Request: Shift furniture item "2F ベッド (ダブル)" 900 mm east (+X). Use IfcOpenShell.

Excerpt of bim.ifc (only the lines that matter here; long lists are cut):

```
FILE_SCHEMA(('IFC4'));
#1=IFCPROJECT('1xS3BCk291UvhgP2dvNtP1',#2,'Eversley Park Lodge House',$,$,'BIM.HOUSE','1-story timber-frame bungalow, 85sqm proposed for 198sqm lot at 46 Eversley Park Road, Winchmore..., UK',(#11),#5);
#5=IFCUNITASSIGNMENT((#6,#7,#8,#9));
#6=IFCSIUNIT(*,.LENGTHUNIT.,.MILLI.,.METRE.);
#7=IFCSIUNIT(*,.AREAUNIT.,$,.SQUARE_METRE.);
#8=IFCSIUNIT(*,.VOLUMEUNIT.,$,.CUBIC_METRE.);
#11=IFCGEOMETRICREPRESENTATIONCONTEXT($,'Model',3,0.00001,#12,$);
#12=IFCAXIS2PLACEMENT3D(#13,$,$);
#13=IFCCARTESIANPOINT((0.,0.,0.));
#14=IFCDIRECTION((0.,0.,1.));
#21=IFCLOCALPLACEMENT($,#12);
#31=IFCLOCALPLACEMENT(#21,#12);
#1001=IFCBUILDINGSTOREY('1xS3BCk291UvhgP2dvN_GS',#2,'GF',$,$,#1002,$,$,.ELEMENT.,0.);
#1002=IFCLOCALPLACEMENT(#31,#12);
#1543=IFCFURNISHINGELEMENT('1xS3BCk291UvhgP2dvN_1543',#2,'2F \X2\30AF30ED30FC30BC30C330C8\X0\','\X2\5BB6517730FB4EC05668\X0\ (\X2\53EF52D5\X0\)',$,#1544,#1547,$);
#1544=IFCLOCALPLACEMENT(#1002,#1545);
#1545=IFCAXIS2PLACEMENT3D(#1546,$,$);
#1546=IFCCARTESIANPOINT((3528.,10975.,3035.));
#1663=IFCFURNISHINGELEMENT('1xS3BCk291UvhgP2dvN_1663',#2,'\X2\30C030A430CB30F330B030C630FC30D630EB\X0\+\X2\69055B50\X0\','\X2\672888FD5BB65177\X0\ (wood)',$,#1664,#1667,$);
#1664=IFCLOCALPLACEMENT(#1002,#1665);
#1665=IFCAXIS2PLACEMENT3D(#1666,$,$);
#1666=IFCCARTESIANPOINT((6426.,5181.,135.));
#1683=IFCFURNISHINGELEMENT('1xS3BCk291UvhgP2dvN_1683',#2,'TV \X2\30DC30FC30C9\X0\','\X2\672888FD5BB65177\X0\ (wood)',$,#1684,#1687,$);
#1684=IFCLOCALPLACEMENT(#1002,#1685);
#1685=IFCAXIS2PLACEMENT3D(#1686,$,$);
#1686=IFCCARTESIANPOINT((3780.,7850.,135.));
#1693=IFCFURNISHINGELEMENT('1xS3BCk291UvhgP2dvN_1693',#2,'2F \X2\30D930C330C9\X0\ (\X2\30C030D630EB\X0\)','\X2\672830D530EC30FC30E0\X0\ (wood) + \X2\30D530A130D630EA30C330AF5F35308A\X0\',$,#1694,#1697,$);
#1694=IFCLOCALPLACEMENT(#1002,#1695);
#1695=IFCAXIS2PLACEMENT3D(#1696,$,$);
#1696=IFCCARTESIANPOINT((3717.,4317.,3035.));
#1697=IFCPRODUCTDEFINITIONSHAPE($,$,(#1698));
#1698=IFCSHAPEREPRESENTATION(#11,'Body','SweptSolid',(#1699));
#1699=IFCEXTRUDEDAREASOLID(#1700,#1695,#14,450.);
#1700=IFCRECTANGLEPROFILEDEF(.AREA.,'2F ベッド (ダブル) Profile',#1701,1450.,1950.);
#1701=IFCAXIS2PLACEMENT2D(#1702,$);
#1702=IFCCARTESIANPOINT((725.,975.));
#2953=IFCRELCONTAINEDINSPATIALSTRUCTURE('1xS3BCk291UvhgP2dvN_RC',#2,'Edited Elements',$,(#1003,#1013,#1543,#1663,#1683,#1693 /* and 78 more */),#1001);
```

```python
import ifcopenshell
import ifcopenshell.api.geometry
import ifcopenshell.util.placement
import ifcopenshell.util.unit

model = ifcopenshell.open("bim.ifc")
unit_scale = ifcopenshell.util.unit.calculate_unit_scale(model)

item = model.by_guid("1xS3BCk291UvhgP2dvN_1693")
matrix = ifcopenshell.util.placement.get_local_placement(item.ObjectPlacement)
matrix[0, 3] += 0.9 / unit_scale
ifcopenshell.api.geometry.edit_object_placement(model, product=item, matrix=matrix, is_si=False)

print(ifcopenshell.util.placement.get_local_placement(item.ObjectPlacement).round(3) + 0.0)

model.write("bim_updated.ifc")
```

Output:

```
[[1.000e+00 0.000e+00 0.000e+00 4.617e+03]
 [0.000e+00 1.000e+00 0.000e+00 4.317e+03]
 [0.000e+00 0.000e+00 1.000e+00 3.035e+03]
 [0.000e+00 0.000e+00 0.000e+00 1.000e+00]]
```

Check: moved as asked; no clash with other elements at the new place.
